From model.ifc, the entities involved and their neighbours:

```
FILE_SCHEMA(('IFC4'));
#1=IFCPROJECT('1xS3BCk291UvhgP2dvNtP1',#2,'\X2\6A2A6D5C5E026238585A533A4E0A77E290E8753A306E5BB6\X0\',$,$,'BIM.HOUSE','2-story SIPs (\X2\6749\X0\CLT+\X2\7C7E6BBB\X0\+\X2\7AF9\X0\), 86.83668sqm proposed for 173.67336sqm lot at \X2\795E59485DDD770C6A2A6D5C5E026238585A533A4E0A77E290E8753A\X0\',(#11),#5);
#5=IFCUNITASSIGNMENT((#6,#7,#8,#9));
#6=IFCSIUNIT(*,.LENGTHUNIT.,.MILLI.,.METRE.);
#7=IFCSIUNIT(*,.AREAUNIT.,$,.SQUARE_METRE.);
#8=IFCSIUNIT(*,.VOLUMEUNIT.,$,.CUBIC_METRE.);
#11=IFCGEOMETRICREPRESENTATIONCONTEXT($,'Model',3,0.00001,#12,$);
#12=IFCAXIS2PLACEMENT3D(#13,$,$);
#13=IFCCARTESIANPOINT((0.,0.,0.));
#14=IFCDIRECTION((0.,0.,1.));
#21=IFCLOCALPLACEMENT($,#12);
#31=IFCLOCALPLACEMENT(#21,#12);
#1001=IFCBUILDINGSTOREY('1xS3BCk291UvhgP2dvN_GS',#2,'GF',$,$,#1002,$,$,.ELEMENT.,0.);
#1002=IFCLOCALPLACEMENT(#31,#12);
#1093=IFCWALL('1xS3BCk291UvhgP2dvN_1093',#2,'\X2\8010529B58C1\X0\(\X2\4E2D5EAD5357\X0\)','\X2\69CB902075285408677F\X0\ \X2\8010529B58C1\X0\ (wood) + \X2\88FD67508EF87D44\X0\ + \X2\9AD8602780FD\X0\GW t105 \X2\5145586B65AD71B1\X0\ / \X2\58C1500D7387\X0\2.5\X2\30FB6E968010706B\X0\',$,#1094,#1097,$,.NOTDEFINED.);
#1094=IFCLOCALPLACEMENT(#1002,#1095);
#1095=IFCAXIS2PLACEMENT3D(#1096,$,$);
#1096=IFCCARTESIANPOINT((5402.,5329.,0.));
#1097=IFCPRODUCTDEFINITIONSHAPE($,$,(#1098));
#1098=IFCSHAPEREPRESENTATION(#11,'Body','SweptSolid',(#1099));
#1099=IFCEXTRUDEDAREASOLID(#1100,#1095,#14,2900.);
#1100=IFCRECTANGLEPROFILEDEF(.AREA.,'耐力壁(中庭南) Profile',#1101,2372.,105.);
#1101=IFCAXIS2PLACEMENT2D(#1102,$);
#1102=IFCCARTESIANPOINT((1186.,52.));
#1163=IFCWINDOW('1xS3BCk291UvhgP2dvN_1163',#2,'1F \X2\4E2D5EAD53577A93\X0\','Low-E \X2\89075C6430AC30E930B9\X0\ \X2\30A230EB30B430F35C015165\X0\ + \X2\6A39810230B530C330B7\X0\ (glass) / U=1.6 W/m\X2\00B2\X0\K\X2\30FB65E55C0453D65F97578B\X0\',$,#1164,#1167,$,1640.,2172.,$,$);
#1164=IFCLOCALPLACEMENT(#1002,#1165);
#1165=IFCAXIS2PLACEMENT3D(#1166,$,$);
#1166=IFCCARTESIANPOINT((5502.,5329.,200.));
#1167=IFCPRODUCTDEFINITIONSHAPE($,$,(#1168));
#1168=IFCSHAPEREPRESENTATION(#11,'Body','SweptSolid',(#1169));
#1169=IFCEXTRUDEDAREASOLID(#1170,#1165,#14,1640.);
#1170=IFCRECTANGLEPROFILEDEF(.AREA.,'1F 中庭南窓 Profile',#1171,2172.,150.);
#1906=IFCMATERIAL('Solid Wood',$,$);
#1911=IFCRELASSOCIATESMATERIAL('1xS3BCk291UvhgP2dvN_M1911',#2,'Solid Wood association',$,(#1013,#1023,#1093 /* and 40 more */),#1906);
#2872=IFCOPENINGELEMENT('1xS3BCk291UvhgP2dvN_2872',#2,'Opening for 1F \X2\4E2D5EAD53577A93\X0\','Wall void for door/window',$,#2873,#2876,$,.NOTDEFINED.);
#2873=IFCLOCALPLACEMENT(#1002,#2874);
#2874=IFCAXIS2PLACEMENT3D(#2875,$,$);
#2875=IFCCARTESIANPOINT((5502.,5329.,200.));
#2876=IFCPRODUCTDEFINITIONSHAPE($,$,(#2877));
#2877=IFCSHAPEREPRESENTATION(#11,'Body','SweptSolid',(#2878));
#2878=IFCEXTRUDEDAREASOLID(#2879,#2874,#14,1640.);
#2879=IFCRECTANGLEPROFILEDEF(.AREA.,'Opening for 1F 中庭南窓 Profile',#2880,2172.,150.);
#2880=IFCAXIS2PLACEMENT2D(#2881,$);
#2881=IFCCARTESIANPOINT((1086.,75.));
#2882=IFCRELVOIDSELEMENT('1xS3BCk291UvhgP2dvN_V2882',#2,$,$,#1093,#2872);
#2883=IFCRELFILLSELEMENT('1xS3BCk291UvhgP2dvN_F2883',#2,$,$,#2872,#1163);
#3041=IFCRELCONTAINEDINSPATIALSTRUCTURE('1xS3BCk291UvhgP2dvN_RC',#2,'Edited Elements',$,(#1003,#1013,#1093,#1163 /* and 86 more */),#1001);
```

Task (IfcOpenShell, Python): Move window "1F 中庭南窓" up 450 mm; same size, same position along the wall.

```python
import numpy as np
import ifcopenshell
import ifcopenshell.api.geometry
import ifcopenshell.util.placement
import ifcopenshell.util.unit

model = ifcopenshell.open("model.ifc")
unit_scale = ifcopenshell.util.unit.calculate_unit_scale(model)

window = model.by_guid("1xS3BCk291UvhgP2dvN_1163")
opening = window.FillsVoids[0].RelatingOpeningElement
dz = 450.0

shift = np.array([0.0, 0.0, dz])
# The window is not placed relative to its opening, so move both.
for product in (opening, window):
    matrix = ifcopenshell.util.placement.get_local_placement(product.ObjectPlacement)
    matrix[:3, 3] += shift
    ifcopenshell.api.geometry.edit_object_placement(model, product=product, matrix=matrix, is_si=False)

print(f"moved by {dz * unit_scale:+.3f} m")

model.write("model_rev.ifc")
```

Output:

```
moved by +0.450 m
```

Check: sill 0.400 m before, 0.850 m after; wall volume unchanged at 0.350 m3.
